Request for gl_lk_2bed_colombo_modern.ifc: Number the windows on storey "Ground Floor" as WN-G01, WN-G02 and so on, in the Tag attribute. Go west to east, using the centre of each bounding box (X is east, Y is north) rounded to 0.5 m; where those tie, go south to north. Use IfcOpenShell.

First a look at what the model holds.

```python
import ifcopenshell
import ifcopenshell.util.element
import ifcopenshell.util.placement

model = ifcopenshell.open("gl_lk_2bed_colombo_modern.ifc")
print(model.schema)
storey = next(s for s in model.by_type("IfcBuildingStorey") if s.Name == "Ground Floor")
windows = [e for e in ifcopenshell.util.element.get_decomposition(storey) if e.is_a("IfcWindow")]
for e in sorted(windows, key=lambda e: e.id()):
    origin = ifcopenshell.util.placement.get_local_placement(e.ObjectPlacement)[:3, 3]
    print(e.id(), e.Tag, e.Name, origin.round(2) + 0.0, sep=" | ")
```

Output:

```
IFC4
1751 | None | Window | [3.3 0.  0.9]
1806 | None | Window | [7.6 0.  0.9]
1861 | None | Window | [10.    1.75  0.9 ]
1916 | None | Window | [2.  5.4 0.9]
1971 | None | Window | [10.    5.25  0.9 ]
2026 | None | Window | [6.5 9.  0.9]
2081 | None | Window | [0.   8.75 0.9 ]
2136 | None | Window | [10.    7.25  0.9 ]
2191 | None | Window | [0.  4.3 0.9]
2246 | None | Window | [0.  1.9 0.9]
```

```python
import ifcopenshell
import ifcopenshell.geom
import ifcopenshell.util.element
import ifcopenshell.util.shape

model = ifcopenshell.open("gl_lk_2bed_colombo_modern.ifc")
settings = ifcopenshell.geom.settings()
settings.set("use-world-coords", True)


def centre(element):
    shape = ifcopenshell.geom.create_shape(settings, element)
    return ifcopenshell.util.shape.get_bbox_centroid(shape.geometry)


storey = next(s for s in model.by_type("IfcBuildingStorey") if s.Name == "Ground Floor")
windows = [e for e in ifcopenshell.util.element.get_decomposition(storey) if e.is_a("IfcWindow")]

# Insertion points can sit at a corner or the storey origin, so sort by the geometry (in metres).
centres = {e: centre(e) for e in windows}
windows.sort(key=lambda e: (round(centres[e][0] / 0.5), centres[e][1]))

for i, e in enumerate(windows, start=1):
    number = f"WN-G{i:02d}"
    e.Tag = number
    print(e.id(), number)

model.write("gl_lk_2bed_colombo_modern_updated.ifc")
```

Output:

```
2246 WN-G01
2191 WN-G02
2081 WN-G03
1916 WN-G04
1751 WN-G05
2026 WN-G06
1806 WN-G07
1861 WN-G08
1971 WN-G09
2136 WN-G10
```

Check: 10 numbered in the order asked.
